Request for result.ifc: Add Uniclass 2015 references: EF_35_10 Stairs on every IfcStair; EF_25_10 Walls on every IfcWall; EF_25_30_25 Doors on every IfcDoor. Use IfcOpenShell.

First a look at what the model holds.

```python
import ifcopenshell

model = ifcopenshell.open("result.ifc")
print(model.schema)
print("classifications:", [c.Name for c in model.by_type("IfcClassification")])
for ifc_class in ("IfcDoor", "IfcRoof", "IfcStair", "IfcWall", "IfcWindow"):
    print(ifc_class, len(model.by_type(ifc_class)))
```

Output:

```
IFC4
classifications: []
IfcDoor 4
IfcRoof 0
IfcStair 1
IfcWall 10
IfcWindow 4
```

```python
import ifcopenshell
import ifcopenshell.api.classification

model = ifcopenshell.open("result.ifc")

system = ifcopenshell.api.classification.add_classification(model, classification="Uniclass 2015")

codes = {
    "IfcStair": ("EF_35_10", "Stairs"),
    "IfcWall": ("EF_25_10", "Walls"),
    "IfcDoor": ("EF_25_30_25", "Doors"),
}
for ifc_class, (code, name) in codes.items():
    products = model.by_type(ifc_class)
    ifcopenshell.api.classification.add_reference(
        model, products=products, classification=system, identification=code, name=name
    )
    print(code, len(products))

model.write("result-out.ifc")
```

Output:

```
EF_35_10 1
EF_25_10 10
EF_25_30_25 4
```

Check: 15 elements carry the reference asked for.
